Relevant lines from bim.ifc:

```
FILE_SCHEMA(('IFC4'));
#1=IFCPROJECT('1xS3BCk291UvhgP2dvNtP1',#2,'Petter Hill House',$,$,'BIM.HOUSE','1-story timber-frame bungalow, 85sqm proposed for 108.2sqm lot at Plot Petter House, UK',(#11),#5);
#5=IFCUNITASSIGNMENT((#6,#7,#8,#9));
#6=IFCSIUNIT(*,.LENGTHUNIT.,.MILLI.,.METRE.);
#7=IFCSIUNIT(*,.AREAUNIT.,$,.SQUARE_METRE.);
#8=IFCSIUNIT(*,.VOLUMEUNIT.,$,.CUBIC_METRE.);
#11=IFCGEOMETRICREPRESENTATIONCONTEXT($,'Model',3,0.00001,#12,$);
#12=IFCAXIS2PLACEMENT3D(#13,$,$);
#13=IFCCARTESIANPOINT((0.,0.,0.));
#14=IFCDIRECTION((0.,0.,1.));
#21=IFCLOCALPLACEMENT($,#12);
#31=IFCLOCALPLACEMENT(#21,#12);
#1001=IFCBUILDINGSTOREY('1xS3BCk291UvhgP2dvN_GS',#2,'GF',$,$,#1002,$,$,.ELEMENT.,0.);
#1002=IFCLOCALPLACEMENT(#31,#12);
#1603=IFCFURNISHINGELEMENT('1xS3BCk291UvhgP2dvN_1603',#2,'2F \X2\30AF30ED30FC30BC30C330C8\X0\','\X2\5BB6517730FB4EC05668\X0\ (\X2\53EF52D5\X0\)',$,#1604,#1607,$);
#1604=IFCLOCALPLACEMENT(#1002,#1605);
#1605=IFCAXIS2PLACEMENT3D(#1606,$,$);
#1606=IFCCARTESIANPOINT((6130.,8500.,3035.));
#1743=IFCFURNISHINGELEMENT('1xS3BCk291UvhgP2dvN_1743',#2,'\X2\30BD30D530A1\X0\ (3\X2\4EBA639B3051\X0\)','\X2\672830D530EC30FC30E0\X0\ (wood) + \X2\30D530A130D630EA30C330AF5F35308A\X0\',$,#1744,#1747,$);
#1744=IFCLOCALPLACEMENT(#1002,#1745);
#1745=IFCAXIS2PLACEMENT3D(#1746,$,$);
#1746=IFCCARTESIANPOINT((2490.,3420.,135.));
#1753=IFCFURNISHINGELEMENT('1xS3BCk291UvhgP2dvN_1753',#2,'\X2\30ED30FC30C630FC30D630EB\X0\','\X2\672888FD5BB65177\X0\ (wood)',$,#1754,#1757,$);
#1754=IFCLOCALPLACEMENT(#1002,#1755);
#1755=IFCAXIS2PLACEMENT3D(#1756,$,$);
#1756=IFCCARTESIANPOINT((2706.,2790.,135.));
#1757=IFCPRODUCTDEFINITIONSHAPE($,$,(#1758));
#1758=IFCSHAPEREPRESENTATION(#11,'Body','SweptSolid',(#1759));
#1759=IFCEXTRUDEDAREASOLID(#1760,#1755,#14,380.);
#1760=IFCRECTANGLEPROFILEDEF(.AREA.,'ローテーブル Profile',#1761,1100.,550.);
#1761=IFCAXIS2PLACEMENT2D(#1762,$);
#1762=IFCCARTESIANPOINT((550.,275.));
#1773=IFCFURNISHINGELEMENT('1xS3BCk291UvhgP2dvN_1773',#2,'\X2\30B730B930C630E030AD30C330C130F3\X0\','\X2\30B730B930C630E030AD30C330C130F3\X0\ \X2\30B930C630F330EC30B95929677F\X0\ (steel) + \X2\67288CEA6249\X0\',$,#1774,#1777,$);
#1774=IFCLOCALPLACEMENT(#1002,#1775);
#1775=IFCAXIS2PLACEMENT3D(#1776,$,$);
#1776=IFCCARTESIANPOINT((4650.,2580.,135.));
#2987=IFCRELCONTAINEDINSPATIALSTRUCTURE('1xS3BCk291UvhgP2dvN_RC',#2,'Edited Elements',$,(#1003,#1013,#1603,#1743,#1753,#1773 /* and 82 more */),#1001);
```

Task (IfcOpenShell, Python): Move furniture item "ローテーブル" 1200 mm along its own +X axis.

```python
import ifcopenshell
import ifcopenshell.api.geometry
import ifcopenshell.util.placement
import ifcopenshell.util.unit

model = ifcopenshell.open("bim.ifc")
unit_scale = ifcopenshell.util.unit.calculate_unit_scale(model)

item = model.by_id(1753)
matrix = ifcopenshell.util.placement.get_local_placement(item.ObjectPlacement)
matrix[:3, 3] += matrix[:3, 0] * 1.2 / unit_scale
ifcopenshell.api.geometry.edit_object_placement(model, product=item, matrix=matrix, is_si=False)

print(ifcopenshell.util.placement.get_local_placement(item.ObjectPlacement).round(3) + 0.0)

model.write("bim-out.ifc")
```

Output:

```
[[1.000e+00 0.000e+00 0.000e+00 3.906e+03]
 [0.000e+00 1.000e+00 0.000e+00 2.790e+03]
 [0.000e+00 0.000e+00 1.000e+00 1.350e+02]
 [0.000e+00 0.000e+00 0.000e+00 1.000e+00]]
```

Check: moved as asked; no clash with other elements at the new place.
